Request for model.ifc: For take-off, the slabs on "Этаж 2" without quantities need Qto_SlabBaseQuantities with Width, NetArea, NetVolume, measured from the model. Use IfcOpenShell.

First a look at what the model holds.

```python
import ifcopenshell
import ifcopenshell.util.element
import ifcopenshell.util.unit

model = ifcopenshell.open("model.ifc")
print(model.schema)
for unit_type in ("LENGTHUNIT", "AREAUNIT", "VOLUMEUNIT"):
    print(unit_type, ifcopenshell.util.unit.calculate_unit_scale(model, unit_type))
storey = next(s for s in model.by_type("IfcBuildingStorey") if s.Name == "Этаж 2")
slabs = [e for e in ifcopenshell.util.element.get_decomposition(storey) if e.is_a("IfcSlab")]
for e in sorted(slabs, key=lambda e: e.id()):
    print(e.id(), e.is_a(), e.Name, list(ifcopenshell.util.element.get_psets(e, qtos_only=True)), sep=" | ")
```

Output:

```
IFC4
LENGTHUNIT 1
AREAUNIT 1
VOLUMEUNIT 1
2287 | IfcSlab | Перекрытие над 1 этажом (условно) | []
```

```python
import ifcopenshell
import ifcopenshell.api.pset
import ifcopenshell.geom
import ifcopenshell.util.element
import ifcopenshell.util.shape
import ifcopenshell.util.unit

model = ifcopenshell.open("model.ifc")
unit_scale = ifcopenshell.util.unit.calculate_unit_scale(model)
area_scale = ifcopenshell.util.unit.calculate_unit_scale(model, "AREAUNIT")
volume_scale = ifcopenshell.util.unit.calculate_unit_scale(model, "VOLUMEUNIT")
settings = ifcopenshell.geom.settings()

storey = next(s for s in model.by_type("IfcBuildingStorey") if s.Name == "Этаж 2")
slabs = [e for e in ifcopenshell.util.element.get_decomposition(storey) if e.is_a("IfcSlab")]

for e in sorted(slabs, key=lambda e: e.id()):
    if ifcopenshell.util.element.get_psets(e, qtos_only=True, should_inherit=False):
        continue
    # Geometry comes back in metres, in the element's own axes.
    shape = ifcopenshell.geom.create_shape(settings, e)
    values = {
        "Width": ifcopenshell.util.shape.get_z(shape.geometry) / unit_scale,
        "NetArea": ifcopenshell.util.shape.get_footprint_area(shape.geometry) / area_scale,
        "NetVolume": ifcopenshell.util.shape.get_volume(shape.geometry) / volume_scale,
    }
    qto = ifcopenshell.api.pset.add_qto(model, product=e, name="Qto_SlabBaseQuantities")
    ifcopenshell.api.pset.edit_qto(model, qto=qto, properties=values)
    print(e.id(), {k: round(v, 3) for k, v in values.items()})

model.write("model_rev.ifc")
```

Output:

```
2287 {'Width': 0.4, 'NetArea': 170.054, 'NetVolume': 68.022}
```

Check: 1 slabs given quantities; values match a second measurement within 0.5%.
